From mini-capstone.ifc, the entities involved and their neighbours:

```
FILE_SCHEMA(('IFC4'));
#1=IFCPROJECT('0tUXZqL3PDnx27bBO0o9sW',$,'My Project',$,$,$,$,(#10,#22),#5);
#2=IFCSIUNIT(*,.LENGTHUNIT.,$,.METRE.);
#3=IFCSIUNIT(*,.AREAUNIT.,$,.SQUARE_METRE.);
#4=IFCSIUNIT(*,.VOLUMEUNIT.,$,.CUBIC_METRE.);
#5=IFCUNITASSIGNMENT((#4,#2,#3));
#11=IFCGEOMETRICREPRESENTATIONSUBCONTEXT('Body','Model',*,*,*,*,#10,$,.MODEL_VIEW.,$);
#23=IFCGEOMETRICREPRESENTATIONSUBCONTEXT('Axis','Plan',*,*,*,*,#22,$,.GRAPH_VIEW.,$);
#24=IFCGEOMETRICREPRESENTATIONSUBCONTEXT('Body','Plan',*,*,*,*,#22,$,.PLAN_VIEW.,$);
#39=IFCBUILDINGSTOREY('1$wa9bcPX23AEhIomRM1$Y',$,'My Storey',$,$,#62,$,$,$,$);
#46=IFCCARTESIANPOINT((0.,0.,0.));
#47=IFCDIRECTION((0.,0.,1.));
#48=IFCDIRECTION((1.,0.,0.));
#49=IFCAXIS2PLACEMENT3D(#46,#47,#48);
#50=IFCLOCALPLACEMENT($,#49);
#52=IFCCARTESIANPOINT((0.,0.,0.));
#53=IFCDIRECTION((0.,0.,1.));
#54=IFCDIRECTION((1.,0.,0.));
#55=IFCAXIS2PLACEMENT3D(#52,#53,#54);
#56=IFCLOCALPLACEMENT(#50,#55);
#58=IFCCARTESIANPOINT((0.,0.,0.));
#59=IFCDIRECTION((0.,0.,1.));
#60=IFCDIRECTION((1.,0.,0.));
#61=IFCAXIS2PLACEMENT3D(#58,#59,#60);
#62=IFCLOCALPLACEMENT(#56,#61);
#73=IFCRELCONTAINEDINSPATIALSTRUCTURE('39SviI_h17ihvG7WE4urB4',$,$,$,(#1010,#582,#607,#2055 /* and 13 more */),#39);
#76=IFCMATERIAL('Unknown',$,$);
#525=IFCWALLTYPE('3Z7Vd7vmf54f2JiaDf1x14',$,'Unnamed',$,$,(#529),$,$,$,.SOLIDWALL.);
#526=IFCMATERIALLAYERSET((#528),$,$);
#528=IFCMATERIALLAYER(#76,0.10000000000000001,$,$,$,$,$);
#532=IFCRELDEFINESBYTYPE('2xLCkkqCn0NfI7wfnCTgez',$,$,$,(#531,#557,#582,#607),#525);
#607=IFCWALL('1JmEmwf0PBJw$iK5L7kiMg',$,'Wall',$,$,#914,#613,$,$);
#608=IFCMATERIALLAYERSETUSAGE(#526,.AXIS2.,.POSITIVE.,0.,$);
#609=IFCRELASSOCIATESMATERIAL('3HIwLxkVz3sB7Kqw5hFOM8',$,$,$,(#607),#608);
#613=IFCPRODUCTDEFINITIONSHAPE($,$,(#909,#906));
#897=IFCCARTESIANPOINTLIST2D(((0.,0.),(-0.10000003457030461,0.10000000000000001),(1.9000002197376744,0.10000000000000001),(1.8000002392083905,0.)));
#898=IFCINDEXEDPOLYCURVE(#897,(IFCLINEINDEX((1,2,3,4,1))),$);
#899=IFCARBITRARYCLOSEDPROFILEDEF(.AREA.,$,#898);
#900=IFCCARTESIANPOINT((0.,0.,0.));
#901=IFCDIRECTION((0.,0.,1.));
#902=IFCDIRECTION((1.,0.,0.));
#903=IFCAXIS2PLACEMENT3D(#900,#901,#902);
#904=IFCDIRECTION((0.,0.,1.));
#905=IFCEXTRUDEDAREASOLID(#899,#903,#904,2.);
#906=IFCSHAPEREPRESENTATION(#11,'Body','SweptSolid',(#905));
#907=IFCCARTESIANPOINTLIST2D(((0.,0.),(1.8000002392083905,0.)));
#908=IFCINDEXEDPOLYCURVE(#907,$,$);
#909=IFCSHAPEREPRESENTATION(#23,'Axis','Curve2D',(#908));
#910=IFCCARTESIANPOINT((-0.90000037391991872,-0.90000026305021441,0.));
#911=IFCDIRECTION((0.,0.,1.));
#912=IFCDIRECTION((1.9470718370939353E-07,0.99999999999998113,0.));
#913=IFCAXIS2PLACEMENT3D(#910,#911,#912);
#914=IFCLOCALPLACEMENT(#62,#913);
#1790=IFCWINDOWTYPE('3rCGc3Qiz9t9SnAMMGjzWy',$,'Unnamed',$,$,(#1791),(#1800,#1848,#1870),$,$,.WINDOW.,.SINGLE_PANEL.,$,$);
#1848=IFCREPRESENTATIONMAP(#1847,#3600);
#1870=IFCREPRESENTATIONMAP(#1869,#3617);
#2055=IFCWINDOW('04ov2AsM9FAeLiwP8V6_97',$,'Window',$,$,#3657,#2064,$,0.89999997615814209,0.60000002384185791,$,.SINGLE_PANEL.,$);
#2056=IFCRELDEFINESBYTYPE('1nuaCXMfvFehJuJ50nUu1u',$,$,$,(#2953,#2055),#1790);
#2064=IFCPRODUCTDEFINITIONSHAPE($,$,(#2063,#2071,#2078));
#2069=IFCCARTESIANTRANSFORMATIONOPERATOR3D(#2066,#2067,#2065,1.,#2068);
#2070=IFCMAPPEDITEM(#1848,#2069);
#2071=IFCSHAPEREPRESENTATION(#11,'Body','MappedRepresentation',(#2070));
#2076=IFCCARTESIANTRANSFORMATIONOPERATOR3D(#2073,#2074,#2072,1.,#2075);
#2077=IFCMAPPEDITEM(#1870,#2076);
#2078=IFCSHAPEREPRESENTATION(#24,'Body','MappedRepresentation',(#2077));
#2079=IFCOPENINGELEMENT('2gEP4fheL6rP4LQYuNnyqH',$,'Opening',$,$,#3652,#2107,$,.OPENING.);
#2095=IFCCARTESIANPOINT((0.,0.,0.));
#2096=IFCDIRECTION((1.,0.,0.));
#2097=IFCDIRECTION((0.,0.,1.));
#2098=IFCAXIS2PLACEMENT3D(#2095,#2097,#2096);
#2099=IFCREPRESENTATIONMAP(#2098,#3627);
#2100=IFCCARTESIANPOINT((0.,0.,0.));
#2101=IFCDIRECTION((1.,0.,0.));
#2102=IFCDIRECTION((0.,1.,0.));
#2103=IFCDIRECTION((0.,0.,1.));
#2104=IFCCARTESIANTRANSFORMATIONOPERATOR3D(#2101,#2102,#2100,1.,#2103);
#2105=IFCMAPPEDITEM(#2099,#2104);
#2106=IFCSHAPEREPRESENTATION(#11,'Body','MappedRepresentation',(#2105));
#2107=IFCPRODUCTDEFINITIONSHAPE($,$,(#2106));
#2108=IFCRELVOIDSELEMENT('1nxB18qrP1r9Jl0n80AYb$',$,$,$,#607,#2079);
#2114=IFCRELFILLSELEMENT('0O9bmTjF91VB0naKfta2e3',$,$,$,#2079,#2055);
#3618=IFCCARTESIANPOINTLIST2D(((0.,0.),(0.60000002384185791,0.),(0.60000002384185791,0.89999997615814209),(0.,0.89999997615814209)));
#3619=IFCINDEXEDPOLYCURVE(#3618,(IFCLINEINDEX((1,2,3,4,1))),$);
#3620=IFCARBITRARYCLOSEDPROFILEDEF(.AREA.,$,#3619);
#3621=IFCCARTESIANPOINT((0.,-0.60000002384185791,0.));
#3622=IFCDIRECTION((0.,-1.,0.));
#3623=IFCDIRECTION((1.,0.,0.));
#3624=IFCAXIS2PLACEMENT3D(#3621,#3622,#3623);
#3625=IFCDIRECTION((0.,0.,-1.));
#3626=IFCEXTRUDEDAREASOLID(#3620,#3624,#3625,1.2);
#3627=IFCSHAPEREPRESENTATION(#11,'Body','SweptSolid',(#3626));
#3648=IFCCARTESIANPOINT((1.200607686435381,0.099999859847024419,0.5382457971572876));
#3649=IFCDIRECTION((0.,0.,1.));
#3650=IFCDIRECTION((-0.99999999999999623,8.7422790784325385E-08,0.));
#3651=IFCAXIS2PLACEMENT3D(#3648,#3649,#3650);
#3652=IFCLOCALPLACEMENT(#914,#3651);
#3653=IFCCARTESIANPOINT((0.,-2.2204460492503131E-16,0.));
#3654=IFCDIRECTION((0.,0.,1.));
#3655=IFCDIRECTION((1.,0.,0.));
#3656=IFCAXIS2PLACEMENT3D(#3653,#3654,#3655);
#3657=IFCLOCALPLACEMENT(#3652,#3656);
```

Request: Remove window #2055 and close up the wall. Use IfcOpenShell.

```python
import ifcopenshell
import ifcopenshell.api.feature
import ifcopenshell.api.root
import ifcopenshell.geom
import ifcopenshell.util.shape

model = ifcopenshell.open("mini-capstone.ifc")
settings = ifcopenshell.geom.settings()


def volume(element):
    """Net volume in cubic metres, openings subtracted."""
    shape = ifcopenshell.geom.create_shape(settings, element)
    return ifcopenshell.util.shape.get_volume(shape.geometry)


window = model.by_guid("04ov2AsM9FAeLiwP8V6_97")
opening = window.FillsVoids[0].RelatingOpeningElement
wall = opening.VoidsElements[0].RelatingBuildingElement
before = volume(wall)

ifcopenshell.api.root.remove_product(model, product=window)
ifcopenshell.api.feature.remove_feature(model, feature=opening)

after = volume(wall)

print(f"wall volume {before:.3f} -> {after:.3f} m3")

model.write("mini-capstone_v2.ifc")
```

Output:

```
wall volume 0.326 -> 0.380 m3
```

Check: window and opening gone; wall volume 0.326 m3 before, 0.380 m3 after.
